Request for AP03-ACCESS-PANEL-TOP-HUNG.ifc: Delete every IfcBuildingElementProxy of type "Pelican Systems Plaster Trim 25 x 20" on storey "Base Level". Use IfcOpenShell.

First a look at what the model holds.

```python
import ifcopenshell
import ifcopenshell.util.element

model = ifcopenshell.open("AP03-ACCESS-PANEL-TOP-HUNG.ifc")
print(model.schema)
storey = next(s for s in model.by_type("IfcBuildingStorey") if s.Name == "Base Level")
proxies = [e for e in ifcopenshell.util.element.get_decomposition(storey) if e.is_a("IfcBuildingElementProxy")]
seen = {}
for e in proxies:
    element_type = ifcopenshell.util.element.get_type(e)
    name = element_type.Name if element_type not in (None, e) else None
    seen[name] = seen.get(name, 0) + 1
for name, count in sorted(seen.items(), key=str):
    print(count, "x", name)
```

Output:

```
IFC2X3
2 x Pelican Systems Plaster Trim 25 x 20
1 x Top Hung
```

```python
import ifcopenshell
import ifcopenshell.api.root
import ifcopenshell.util.element

model = ifcopenshell.open("AP03-ACCESS-PANEL-TOP-HUNG.ifc")

storey = next(s for s in model.by_type("IfcBuildingStorey") if s.Name == "Base Level")
proxies = [e for e in ifcopenshell.util.element.get_decomposition(storey) if e.is_a("IfcBuildingElementProxy")]
targets = [e for e in proxies if (t := ifcopenshell.util.element.get_type(e)) not in (None, e) and t.Name == "Pelican Systems Plaster Trim 25 x 20"]

for e in targets:
    ifcopenshell.api.root.remove_product(model, product=e)
print(len(targets), "removed")

model.write("AP03-ACCESS-PANEL-TOP-HUNG_v2.ifc")
```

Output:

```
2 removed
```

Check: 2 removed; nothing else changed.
